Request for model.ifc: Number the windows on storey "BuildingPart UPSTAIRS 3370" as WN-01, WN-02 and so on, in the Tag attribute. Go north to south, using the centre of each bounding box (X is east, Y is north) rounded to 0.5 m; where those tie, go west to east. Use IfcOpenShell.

First a look at what the model holds.

```python
import ifcopenshell
import ifcopenshell.util.element
import ifcopenshell.util.placement

model = ifcopenshell.open("model.ifc")
print(model.schema)
storey = next(s for s in model.by_type("IfcBuildingStorey") if s.Name == "BuildingPart UPSTAIRS 3370")
windows = [e for e in ifcopenshell.util.element.get_decomposition(storey) if e.is_a("IfcWindow")]
for e in sorted(windows, key=lambda e: e.id()):
    origin = ifcopenshell.util.placement.get_local_placement(e.ObjectPlacement)[:3, 3]
    print(e.id(), e.Tag, e.Name, origin.round(2) + 0.0, sep=" | ")
```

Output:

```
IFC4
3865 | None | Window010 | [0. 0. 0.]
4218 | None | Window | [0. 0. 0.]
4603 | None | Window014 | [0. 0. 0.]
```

```python
import ifcopenshell
import ifcopenshell.geom
import ifcopenshell.util.element
import ifcopenshell.util.shape

model = ifcopenshell.open("model.ifc")
settings = ifcopenshell.geom.settings()
settings.set("use-world-coords", True)


def centre(element):
    shape = ifcopenshell.geom.create_shape(settings, element)
    return ifcopenshell.util.shape.get_bbox_centroid(shape.geometry)


storey = next(s for s in model.by_type("IfcBuildingStorey") if s.Name == "BuildingPart UPSTAIRS 3370")
windows = [e for e in ifcopenshell.util.element.get_decomposition(storey) if e.is_a("IfcWindow")]

# Insertion points can sit at a corner or the storey origin, so sort by the geometry (in metres).
centres = {e: centre(e) for e in windows}
windows.sort(key=lambda e: (-round(centres[e][1] / 0.5), centres[e][0]))

for i, e in enumerate(windows, start=1):
    number = f"WN-{i:02d}"
    e.Tag = number
    print(e.id(), number)

model.write("model_updated.ifc")
```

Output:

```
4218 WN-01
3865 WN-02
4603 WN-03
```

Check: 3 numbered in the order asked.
